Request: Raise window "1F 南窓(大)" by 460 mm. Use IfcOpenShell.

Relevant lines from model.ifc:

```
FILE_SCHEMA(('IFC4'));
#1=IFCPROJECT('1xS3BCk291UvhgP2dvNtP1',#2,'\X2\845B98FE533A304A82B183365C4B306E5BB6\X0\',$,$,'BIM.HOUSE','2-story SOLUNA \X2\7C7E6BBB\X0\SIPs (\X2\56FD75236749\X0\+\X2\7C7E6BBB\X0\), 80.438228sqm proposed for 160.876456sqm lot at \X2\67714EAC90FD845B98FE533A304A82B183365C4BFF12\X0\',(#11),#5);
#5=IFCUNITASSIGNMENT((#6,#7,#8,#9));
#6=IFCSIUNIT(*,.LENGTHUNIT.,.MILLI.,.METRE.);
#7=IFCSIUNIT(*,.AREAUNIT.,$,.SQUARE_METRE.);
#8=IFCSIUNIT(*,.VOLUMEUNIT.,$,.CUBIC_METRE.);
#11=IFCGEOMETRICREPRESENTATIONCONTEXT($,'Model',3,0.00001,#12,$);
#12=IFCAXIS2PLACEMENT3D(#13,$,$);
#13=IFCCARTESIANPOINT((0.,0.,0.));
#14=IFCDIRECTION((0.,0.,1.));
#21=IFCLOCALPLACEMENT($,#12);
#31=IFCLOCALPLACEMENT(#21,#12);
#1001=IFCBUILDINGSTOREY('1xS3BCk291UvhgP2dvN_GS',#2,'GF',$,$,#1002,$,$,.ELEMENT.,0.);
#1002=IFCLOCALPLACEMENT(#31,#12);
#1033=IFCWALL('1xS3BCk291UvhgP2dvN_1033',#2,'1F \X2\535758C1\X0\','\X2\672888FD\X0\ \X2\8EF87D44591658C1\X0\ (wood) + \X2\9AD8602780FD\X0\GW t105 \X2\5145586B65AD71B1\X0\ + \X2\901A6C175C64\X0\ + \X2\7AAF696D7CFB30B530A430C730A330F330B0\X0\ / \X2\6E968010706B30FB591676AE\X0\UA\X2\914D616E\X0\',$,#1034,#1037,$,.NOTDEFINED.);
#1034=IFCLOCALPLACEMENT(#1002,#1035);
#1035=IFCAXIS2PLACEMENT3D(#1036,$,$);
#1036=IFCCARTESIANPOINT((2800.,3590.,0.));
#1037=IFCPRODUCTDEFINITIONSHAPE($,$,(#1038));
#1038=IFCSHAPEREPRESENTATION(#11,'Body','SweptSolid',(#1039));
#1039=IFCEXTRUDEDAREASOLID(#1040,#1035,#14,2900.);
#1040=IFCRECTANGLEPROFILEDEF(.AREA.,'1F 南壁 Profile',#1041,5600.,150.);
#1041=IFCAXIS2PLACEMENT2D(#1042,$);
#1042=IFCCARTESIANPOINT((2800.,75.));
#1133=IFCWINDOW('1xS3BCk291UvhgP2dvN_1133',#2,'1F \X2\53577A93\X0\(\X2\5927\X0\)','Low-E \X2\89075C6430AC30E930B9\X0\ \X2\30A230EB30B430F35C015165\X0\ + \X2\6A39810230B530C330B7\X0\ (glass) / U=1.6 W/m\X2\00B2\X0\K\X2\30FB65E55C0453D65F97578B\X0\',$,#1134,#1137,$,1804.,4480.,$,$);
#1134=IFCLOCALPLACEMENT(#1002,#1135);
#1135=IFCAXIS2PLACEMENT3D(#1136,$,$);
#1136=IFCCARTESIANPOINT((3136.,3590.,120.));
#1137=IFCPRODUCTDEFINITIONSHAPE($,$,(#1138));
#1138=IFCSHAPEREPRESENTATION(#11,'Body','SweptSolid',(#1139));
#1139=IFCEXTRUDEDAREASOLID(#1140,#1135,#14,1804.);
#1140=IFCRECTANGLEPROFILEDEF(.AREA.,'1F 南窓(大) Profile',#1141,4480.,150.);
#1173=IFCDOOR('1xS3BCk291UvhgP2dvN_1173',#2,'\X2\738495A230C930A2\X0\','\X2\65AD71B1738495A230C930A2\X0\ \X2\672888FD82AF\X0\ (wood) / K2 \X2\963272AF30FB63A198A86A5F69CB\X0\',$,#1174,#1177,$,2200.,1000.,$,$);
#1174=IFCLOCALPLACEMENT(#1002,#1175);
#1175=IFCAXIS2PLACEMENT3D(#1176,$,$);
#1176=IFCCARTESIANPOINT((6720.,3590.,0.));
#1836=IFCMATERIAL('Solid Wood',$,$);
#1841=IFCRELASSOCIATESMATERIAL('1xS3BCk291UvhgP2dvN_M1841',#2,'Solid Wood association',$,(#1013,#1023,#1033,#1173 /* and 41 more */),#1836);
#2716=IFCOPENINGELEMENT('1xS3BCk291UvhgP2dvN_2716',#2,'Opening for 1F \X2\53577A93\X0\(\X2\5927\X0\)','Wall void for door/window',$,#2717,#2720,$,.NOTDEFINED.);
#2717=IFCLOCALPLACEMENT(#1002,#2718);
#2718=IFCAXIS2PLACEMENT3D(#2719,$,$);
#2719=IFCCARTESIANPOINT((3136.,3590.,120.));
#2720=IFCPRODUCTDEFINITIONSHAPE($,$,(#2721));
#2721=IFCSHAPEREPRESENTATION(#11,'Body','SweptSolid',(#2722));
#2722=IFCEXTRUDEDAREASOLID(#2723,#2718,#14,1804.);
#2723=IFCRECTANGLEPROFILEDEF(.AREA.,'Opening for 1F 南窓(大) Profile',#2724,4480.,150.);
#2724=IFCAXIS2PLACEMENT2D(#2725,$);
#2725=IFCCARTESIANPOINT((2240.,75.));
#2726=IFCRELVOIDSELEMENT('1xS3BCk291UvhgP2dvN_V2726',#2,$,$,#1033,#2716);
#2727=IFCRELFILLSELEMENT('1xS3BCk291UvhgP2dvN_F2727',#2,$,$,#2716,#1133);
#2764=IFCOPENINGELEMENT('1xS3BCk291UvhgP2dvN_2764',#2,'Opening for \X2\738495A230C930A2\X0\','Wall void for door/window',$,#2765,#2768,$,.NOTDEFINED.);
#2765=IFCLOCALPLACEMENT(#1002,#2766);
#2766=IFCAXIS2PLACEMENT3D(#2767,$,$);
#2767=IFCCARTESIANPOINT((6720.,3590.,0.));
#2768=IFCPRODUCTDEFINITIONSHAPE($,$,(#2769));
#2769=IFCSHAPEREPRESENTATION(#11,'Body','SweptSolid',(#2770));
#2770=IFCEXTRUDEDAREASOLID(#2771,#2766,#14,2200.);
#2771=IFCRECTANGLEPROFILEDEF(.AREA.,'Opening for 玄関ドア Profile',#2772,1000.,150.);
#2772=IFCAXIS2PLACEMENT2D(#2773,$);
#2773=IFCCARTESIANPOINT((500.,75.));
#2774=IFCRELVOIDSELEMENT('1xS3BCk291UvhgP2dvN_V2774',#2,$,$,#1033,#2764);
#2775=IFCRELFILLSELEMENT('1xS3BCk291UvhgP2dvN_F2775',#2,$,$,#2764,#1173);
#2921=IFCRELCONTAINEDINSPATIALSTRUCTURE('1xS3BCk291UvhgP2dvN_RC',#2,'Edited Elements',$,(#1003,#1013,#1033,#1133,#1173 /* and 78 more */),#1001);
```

```python
import numpy as np
import ifcopenshell
import ifcopenshell.api.geometry
import ifcopenshell.util.placement
import ifcopenshell.util.unit

model = ifcopenshell.open("model.ifc")
unit_scale = ifcopenshell.util.unit.calculate_unit_scale(model)

window = model.by_id(1133)
opening = window.FillsVoids[0].RelatingOpeningElement
dz = 0.46 / unit_scale

shift = np.array([0.0, 0.0, dz])
# The window is not placed relative to its opening, so move both.
for product in (opening, window):
    matrix = ifcopenshell.util.placement.get_local_placement(product.ObjectPlacement)
    matrix[:3, 3] += shift
    ifcopenshell.api.geometry.edit_object_placement(model, product=product, matrix=matrix, is_si=False)

print(f"moved by {dz * unit_scale:+.3f} m")

model.write("model-out.ifc")
```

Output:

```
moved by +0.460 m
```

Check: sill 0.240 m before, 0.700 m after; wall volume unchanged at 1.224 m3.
